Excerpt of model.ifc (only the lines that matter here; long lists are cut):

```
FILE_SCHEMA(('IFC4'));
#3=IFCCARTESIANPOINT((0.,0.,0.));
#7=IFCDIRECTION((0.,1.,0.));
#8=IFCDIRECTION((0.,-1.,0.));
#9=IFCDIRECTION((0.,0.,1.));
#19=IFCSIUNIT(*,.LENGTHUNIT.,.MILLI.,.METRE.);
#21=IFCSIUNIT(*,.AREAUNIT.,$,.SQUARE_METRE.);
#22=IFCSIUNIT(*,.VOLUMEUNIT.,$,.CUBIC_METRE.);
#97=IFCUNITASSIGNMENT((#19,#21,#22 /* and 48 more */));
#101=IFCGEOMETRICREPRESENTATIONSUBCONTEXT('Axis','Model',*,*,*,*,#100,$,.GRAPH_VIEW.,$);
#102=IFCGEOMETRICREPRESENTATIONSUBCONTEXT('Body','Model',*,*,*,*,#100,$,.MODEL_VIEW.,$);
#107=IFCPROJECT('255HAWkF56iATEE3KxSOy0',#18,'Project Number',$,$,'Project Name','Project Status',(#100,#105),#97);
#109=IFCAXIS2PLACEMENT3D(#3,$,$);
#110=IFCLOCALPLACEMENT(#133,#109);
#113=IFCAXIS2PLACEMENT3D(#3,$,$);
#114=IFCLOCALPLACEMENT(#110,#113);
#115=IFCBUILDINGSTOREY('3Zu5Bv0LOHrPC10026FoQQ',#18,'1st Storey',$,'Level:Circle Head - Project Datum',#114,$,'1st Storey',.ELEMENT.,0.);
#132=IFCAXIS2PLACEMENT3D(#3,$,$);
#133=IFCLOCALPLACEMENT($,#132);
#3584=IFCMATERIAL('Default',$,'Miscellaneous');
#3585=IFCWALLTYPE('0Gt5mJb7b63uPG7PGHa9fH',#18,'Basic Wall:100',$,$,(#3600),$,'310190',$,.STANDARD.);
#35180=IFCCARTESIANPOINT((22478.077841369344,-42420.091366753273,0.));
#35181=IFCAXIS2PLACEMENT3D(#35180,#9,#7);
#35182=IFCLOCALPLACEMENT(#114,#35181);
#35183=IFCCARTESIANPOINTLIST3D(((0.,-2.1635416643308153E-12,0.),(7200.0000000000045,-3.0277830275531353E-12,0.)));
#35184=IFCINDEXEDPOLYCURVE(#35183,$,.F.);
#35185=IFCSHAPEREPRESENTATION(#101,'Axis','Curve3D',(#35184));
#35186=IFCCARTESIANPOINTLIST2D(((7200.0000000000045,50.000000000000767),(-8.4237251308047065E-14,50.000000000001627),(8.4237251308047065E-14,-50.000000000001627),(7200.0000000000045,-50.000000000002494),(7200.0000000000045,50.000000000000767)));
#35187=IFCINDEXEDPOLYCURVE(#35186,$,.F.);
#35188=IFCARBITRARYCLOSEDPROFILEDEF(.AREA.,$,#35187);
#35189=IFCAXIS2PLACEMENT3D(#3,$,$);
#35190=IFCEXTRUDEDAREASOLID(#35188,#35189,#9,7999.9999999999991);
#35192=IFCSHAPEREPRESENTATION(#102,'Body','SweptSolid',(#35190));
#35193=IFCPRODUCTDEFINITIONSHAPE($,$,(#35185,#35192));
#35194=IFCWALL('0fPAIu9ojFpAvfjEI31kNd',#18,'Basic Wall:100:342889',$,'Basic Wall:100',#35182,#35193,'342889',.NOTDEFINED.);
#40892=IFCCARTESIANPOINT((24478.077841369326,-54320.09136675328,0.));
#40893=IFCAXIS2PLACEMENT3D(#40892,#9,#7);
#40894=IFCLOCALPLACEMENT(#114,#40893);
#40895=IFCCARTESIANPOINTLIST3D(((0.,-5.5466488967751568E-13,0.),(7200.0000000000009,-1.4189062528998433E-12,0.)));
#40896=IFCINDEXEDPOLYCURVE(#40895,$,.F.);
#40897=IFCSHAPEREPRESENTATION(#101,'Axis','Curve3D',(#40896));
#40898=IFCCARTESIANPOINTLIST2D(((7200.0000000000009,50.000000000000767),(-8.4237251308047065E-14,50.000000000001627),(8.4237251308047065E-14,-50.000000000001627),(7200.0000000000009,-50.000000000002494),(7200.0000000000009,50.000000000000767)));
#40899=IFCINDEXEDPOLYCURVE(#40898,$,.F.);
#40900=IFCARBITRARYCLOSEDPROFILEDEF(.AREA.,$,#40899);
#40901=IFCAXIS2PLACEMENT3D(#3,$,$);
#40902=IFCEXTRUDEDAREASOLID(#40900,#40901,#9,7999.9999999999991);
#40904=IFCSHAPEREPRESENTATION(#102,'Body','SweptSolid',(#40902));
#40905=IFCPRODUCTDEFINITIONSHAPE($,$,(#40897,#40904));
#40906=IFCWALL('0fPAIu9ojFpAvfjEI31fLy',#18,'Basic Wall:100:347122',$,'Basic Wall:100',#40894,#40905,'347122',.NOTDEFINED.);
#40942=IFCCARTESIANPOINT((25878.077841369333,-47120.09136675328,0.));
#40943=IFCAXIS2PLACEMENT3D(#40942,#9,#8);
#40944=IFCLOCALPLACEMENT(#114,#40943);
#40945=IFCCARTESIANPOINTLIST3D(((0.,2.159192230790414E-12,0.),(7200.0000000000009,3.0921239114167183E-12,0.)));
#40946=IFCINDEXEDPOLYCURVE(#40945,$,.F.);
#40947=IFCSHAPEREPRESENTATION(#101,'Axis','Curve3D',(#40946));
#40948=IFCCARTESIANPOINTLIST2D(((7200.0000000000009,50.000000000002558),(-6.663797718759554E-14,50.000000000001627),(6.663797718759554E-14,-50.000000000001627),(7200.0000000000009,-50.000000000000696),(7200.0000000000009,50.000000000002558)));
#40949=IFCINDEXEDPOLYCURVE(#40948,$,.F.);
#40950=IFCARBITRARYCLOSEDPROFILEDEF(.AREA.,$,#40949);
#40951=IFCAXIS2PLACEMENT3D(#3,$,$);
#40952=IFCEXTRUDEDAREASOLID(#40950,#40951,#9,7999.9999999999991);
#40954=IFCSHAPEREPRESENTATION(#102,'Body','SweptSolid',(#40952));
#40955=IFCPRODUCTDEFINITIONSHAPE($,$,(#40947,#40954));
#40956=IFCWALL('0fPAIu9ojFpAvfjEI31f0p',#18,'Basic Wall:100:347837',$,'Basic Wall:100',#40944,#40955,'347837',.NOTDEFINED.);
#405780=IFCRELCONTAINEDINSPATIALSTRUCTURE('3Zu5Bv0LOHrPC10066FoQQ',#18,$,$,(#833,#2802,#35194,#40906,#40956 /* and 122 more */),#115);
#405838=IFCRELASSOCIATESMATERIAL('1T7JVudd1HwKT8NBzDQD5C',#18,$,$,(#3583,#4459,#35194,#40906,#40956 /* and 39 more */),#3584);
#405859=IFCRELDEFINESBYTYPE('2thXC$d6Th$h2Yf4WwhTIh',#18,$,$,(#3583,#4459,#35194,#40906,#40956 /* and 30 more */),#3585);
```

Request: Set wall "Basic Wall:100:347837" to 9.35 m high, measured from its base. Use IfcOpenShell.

```python
import ifcopenshell
import ifcopenshell.geom
import ifcopenshell.util.representation
import ifcopenshell.util.shape
import ifcopenshell.util.unit

model = ifcopenshell.open("model.ifc")
unit_scale = ifcopenshell.util.unit.calculate_unit_scale(model)
settings = ifcopenshell.geom.settings()


def volume(element):
    """Net volume in cubic metres, openings subtracted."""
    shape = ifcopenshell.geom.create_shape(settings, element)
    return ifcopenshell.util.shape.get_volume(shape.geometry)


wall = model.by_guid("0fPAIu9ojFpAvfjEI31f0p")
before = volume(wall)

body = ifcopenshell.util.representation.get_representation(wall, "Model", "Body")
solid = body.Items[0]
old_height = solid.Depth
solid.Depth = 9.35 / unit_scale
after = volume(wall)

print(f"height {old_height:g} -> {solid.Depth:g}, volume {before:.3f} -> {after:.3f} m3")

model.write("model_edited.ifc")
```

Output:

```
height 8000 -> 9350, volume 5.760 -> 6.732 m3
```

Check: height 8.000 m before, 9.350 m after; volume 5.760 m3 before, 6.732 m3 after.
